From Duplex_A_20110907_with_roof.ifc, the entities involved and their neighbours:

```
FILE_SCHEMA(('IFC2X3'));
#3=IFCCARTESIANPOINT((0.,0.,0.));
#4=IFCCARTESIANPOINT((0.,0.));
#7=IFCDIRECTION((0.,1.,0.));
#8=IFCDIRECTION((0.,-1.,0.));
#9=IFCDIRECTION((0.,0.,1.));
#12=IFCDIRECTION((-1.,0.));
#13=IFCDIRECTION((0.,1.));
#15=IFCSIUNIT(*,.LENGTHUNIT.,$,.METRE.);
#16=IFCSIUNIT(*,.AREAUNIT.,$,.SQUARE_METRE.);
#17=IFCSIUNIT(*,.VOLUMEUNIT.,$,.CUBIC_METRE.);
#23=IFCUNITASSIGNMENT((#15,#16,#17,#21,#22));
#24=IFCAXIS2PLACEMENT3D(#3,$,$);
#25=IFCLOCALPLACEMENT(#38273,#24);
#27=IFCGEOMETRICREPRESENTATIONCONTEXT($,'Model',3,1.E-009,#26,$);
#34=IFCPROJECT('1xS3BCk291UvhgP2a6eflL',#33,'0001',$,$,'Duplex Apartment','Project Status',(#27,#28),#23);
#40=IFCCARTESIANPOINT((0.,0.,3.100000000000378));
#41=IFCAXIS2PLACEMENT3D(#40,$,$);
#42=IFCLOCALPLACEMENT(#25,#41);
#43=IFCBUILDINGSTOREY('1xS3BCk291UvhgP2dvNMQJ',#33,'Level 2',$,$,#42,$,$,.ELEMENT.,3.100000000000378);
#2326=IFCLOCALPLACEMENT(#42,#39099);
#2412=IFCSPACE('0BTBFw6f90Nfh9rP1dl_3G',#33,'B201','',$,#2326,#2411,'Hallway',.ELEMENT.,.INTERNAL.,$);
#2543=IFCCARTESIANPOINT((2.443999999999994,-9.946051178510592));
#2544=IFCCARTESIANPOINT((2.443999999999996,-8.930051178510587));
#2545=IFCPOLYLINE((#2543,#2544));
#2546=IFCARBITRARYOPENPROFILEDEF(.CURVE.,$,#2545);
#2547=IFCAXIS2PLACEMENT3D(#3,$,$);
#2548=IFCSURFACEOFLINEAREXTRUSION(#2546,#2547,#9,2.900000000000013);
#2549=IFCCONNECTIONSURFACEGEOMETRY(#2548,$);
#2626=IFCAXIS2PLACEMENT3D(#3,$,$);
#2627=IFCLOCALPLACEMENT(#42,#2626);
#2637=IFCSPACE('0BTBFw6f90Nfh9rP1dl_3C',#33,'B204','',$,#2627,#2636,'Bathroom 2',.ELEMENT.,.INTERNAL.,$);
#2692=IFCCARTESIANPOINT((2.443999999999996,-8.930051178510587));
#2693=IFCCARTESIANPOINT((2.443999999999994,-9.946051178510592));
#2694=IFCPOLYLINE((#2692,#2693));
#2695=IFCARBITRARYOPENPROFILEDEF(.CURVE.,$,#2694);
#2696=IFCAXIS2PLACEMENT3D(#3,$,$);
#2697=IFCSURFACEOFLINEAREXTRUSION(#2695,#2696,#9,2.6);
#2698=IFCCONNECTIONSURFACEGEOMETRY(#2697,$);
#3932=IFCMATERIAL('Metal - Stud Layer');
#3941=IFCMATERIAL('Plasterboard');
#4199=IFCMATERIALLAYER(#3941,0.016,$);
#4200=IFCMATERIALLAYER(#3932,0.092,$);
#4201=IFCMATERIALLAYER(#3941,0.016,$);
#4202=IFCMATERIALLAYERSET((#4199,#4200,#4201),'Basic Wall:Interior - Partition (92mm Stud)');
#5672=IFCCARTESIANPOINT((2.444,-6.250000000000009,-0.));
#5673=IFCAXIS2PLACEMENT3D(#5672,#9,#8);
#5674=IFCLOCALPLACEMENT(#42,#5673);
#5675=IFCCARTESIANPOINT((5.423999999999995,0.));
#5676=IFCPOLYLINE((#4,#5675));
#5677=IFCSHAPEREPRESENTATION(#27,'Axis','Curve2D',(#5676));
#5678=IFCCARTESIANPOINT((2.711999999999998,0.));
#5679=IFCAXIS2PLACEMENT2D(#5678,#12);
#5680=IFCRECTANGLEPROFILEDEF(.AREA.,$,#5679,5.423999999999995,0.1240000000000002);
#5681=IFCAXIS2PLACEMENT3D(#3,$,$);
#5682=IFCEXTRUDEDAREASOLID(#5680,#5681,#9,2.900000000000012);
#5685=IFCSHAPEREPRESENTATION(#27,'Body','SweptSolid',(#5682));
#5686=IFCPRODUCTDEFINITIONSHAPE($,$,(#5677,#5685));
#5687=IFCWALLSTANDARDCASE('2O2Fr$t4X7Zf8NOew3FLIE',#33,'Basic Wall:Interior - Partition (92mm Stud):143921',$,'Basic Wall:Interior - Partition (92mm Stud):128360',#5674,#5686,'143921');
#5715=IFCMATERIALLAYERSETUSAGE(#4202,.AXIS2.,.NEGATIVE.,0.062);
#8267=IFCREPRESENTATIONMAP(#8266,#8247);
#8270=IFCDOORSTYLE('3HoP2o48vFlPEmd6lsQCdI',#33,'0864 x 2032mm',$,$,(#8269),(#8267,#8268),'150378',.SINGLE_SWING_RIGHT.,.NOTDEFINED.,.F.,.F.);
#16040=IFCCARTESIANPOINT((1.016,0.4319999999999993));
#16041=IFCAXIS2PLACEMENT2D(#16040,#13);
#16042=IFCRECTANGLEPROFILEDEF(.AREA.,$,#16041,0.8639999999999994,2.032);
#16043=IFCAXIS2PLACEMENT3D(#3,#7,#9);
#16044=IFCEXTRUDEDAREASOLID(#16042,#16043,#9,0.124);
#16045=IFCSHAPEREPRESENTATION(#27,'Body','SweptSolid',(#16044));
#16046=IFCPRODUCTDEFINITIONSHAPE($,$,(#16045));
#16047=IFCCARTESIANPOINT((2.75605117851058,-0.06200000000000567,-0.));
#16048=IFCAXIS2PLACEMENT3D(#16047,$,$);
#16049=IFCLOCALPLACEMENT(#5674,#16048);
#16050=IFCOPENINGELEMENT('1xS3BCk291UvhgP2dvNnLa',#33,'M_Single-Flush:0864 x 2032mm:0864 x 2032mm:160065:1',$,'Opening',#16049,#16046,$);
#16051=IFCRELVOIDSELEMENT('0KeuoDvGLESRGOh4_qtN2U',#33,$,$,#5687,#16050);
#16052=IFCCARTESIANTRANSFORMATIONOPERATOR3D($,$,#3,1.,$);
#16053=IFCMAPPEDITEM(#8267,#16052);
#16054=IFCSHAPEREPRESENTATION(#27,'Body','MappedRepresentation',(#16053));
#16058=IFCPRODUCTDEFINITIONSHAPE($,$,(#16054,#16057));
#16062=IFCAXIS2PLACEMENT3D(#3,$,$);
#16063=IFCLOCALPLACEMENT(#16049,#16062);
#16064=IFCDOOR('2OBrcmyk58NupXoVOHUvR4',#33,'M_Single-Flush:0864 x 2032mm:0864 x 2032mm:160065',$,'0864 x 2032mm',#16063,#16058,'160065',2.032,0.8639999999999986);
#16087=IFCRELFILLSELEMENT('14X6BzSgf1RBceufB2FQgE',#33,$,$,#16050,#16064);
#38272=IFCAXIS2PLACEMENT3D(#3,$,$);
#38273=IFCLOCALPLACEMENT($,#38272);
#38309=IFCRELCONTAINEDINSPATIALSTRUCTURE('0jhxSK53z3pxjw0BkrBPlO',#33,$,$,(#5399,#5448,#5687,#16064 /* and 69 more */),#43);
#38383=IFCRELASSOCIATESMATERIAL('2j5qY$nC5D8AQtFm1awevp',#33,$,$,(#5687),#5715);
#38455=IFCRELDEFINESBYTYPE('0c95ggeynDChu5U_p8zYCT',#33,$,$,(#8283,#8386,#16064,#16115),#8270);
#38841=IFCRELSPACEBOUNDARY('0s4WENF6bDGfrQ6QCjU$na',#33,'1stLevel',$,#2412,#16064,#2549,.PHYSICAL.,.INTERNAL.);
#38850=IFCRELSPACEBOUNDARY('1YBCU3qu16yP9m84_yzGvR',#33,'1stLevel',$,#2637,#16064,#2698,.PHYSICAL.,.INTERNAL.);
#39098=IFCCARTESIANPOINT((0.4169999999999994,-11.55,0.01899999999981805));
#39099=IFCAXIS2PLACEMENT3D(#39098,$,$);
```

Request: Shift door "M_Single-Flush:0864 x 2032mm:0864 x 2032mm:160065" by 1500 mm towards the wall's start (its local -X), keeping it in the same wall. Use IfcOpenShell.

```python
import numpy as np
import ifcopenshell
import ifcopenshell.api.geometry
import ifcopenshell.util.placement

model = ifcopenshell.open("Duplex_A_20110907_with_roof.ifc")

door = model.by_id(16064)
opening = door.FillsVoids[0].RelatingOpeningElement
wall = opening.VoidsElements[0].RelatingBuildingElement

wall_matrix = ifcopenshell.util.placement.get_local_placement(wall.ObjectPlacement)
shift = wall_matrix[:3, 0] * -1.5
before = ifcopenshell.util.placement.get_local_placement(door.ObjectPlacement)[:3, 3].copy()

# The door is placed relative to its opening, so it follows when the opening moves.
matrix = ifcopenshell.util.placement.get_local_placement(opening.ObjectPlacement)
matrix[:3, 3] += shift
ifcopenshell.api.geometry.edit_object_placement(
    model, product=opening, matrix=matrix, is_si=False, should_transform_children=True
)

# Space boundary surfaces are stored in each space's coordinates; move them too.
for rel in door.ProvidesBoundaries:
    if not rel.ConnectionGeometry:
        continue
    surface = rel.ConnectionGeometry.SurfaceOnRelatingElement
    space_matrix = ifcopenshell.util.placement.get_local_placement(rel.RelatingSpace.ObjectPlacement)
    point = np.array(surface.Position.Location.Coordinates) + space_matrix[:3, :3].T @ shift
    surface.Position = model.createIfcAxis2Placement3D(
        model.createIfcCartesianPoint(point.tolist()), surface.Position.Axis, surface.Position.RefDirection
    )

after = ifcopenshell.util.placement.get_local_placement(door.ObjectPlacement)[:3, 3]
print("door moved by", (after - before).round(3) + 0.0)

model.write("Duplex_A_20110907_with_roof_rev.ifc")
```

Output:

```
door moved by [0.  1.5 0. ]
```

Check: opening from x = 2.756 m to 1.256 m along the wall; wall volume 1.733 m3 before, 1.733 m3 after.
